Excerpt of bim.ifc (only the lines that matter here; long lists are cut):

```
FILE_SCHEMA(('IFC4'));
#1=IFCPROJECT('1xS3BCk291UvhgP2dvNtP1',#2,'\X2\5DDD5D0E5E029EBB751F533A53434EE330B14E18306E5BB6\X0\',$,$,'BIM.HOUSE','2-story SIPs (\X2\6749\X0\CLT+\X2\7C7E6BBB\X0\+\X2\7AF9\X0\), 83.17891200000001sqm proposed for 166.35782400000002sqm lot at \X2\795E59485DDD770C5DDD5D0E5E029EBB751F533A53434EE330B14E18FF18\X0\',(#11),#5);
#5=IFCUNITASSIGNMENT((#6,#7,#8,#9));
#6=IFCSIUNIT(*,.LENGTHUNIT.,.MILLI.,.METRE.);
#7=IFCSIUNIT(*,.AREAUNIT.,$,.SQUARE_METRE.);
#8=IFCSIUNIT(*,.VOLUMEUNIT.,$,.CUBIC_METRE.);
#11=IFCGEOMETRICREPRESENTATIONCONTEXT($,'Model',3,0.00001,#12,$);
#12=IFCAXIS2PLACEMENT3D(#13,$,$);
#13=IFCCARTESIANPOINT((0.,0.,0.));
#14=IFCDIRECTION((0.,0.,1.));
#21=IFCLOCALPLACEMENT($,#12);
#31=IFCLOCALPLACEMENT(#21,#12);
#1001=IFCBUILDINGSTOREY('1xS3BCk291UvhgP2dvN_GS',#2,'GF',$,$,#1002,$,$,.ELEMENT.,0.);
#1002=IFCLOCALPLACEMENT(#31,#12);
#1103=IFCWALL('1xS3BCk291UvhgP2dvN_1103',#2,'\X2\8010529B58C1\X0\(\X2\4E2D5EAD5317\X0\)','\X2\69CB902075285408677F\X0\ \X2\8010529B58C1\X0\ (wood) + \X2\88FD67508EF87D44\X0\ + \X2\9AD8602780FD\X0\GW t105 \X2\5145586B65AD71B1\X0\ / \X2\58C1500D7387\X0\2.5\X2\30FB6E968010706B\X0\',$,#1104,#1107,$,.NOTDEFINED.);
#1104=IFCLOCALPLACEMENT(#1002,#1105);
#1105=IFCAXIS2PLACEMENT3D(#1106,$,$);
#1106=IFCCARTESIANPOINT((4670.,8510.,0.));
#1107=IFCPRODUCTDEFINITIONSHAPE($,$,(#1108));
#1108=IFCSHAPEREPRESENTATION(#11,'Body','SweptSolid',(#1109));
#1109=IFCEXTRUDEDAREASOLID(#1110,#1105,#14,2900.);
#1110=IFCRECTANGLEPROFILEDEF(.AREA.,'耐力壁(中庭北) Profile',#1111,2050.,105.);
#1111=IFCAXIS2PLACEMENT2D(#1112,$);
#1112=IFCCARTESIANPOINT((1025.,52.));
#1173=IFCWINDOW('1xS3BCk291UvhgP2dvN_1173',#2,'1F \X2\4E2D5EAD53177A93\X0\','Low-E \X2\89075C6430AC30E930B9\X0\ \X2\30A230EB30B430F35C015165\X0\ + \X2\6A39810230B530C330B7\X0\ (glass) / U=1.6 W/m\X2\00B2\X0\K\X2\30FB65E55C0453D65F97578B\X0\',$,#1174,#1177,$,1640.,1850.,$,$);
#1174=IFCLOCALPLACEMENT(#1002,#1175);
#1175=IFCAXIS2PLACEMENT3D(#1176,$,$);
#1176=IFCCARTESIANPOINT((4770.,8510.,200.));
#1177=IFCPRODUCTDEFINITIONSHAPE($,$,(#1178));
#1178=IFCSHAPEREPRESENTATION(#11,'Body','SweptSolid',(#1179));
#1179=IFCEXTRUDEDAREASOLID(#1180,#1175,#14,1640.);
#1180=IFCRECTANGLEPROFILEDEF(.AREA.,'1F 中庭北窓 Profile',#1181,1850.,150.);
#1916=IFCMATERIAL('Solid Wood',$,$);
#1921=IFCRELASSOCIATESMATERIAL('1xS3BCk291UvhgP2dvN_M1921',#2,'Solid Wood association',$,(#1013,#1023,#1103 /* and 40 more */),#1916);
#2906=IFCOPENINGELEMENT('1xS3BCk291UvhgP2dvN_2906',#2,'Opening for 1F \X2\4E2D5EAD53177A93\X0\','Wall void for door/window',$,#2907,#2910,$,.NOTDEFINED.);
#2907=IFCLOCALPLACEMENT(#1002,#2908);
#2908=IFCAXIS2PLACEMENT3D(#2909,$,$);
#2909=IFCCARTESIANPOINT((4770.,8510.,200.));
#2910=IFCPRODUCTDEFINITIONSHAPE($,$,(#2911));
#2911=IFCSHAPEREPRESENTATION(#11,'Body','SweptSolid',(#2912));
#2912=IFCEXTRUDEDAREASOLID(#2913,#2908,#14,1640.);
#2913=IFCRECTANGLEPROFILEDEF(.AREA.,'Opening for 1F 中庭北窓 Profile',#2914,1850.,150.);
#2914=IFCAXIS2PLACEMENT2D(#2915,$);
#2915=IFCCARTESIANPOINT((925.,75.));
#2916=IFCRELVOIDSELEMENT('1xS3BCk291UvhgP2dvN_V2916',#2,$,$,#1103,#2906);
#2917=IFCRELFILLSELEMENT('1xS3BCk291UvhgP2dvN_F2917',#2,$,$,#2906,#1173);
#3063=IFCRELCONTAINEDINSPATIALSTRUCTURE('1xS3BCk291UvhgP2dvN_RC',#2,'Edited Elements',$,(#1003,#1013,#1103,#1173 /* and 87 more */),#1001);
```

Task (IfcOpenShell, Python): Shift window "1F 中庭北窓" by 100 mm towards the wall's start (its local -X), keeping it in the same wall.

```python
import ifcopenshell
import ifcopenshell.api.geometry
import ifcopenshell.util.placement

model = ifcopenshell.open("bim.ifc")

window = model.by_guid("1xS3BCk291UvhgP2dvN_1173")
opening = window.FillsVoids[0].RelatingOpeningElement
wall = opening.VoidsElements[0].RelatingBuildingElement

wall_matrix = ifcopenshell.util.placement.get_local_placement(wall.ObjectPlacement)
shift = wall_matrix[:3, 0] * -100.0
before = ifcopenshell.util.placement.get_local_placement(window.ObjectPlacement)[:3, 3].copy()

# The window is not placed relative to its opening, so move both.
for product in (opening, window):
    matrix = ifcopenshell.util.placement.get_local_placement(product.ObjectPlacement)
    matrix[:3, 3] += shift
    ifcopenshell.api.geometry.edit_object_placement(model, product=product, matrix=matrix, is_si=False)

after = ifcopenshell.util.placement.get_local_placement(window.ObjectPlacement)[:3, 3]
print("window moved by", (after - before).round(3) + 0.0)

model.write("bim_edited.ifc")
```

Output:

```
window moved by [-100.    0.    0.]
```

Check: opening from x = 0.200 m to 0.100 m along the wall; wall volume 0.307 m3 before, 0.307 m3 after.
